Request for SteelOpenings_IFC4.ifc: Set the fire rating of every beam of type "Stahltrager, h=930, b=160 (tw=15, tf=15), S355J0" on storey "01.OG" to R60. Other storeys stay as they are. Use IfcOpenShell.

First a look at what the model holds.

```python
import ifcopenshell
import ifcopenshell.util.element

model = ifcopenshell.open("SteelOpenings_IFC4.ifc")
print(model.schema)
storey = next(s for s in model.by_type("IfcBuildingStorey") if s.Name == "01.OG")
beams = [e for e in ifcopenshell.util.element.get_decomposition(storey) if e.is_a("IfcBeam")]
seen = {}
for e in beams:
    element_type = ifcopenshell.util.element.get_type(e)
    key = (element_type.Name if element_type != e and element_type else None, ifcopenshell.util.element.get_pset(e, "Pset_BeamCommon", "FireRating"))
    seen[key] = seen.get(key, 0) + 1
for (name, value), count in sorted(seen.items(), key=str):
    print(count, "x", name, "|", value)
```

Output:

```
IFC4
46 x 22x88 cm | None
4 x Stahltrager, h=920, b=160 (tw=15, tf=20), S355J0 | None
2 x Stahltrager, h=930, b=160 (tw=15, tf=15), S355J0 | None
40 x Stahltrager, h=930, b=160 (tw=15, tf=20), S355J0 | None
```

```python
import ifcopenshell
import ifcopenshell.api.pset
import ifcopenshell.util.element

model = ifcopenshell.open("SteelOpenings_IFC4.ifc")

storey = next(s for s in model.by_type("IfcBuildingStorey") if s.Name == "01.OG")
beams = [e for e in ifcopenshell.util.element.get_decomposition(storey) if e.is_a("IfcBeam")]

count = 0
for e in beams:
    element_type = ifcopenshell.util.element.get_type(e)
    if element_type in (None, e) or element_type.Name != "Stahltrager, h=930, b=160 (tw=15, tf=15), S355J0":
        continue
    # add_pset returns the element's existing set when there is one.
    pset = ifcopenshell.api.pset.add_pset(model, product=e, name="Pset_BeamCommon")
    ifcopenshell.api.pset.edit_pset(model, pset=pset, properties={"FireRating": "R60"})
    count += 1

print(count, "beams updated")

model.write("SteelOpenings_IFC4-out.ifc")
```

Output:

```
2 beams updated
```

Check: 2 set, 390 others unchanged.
